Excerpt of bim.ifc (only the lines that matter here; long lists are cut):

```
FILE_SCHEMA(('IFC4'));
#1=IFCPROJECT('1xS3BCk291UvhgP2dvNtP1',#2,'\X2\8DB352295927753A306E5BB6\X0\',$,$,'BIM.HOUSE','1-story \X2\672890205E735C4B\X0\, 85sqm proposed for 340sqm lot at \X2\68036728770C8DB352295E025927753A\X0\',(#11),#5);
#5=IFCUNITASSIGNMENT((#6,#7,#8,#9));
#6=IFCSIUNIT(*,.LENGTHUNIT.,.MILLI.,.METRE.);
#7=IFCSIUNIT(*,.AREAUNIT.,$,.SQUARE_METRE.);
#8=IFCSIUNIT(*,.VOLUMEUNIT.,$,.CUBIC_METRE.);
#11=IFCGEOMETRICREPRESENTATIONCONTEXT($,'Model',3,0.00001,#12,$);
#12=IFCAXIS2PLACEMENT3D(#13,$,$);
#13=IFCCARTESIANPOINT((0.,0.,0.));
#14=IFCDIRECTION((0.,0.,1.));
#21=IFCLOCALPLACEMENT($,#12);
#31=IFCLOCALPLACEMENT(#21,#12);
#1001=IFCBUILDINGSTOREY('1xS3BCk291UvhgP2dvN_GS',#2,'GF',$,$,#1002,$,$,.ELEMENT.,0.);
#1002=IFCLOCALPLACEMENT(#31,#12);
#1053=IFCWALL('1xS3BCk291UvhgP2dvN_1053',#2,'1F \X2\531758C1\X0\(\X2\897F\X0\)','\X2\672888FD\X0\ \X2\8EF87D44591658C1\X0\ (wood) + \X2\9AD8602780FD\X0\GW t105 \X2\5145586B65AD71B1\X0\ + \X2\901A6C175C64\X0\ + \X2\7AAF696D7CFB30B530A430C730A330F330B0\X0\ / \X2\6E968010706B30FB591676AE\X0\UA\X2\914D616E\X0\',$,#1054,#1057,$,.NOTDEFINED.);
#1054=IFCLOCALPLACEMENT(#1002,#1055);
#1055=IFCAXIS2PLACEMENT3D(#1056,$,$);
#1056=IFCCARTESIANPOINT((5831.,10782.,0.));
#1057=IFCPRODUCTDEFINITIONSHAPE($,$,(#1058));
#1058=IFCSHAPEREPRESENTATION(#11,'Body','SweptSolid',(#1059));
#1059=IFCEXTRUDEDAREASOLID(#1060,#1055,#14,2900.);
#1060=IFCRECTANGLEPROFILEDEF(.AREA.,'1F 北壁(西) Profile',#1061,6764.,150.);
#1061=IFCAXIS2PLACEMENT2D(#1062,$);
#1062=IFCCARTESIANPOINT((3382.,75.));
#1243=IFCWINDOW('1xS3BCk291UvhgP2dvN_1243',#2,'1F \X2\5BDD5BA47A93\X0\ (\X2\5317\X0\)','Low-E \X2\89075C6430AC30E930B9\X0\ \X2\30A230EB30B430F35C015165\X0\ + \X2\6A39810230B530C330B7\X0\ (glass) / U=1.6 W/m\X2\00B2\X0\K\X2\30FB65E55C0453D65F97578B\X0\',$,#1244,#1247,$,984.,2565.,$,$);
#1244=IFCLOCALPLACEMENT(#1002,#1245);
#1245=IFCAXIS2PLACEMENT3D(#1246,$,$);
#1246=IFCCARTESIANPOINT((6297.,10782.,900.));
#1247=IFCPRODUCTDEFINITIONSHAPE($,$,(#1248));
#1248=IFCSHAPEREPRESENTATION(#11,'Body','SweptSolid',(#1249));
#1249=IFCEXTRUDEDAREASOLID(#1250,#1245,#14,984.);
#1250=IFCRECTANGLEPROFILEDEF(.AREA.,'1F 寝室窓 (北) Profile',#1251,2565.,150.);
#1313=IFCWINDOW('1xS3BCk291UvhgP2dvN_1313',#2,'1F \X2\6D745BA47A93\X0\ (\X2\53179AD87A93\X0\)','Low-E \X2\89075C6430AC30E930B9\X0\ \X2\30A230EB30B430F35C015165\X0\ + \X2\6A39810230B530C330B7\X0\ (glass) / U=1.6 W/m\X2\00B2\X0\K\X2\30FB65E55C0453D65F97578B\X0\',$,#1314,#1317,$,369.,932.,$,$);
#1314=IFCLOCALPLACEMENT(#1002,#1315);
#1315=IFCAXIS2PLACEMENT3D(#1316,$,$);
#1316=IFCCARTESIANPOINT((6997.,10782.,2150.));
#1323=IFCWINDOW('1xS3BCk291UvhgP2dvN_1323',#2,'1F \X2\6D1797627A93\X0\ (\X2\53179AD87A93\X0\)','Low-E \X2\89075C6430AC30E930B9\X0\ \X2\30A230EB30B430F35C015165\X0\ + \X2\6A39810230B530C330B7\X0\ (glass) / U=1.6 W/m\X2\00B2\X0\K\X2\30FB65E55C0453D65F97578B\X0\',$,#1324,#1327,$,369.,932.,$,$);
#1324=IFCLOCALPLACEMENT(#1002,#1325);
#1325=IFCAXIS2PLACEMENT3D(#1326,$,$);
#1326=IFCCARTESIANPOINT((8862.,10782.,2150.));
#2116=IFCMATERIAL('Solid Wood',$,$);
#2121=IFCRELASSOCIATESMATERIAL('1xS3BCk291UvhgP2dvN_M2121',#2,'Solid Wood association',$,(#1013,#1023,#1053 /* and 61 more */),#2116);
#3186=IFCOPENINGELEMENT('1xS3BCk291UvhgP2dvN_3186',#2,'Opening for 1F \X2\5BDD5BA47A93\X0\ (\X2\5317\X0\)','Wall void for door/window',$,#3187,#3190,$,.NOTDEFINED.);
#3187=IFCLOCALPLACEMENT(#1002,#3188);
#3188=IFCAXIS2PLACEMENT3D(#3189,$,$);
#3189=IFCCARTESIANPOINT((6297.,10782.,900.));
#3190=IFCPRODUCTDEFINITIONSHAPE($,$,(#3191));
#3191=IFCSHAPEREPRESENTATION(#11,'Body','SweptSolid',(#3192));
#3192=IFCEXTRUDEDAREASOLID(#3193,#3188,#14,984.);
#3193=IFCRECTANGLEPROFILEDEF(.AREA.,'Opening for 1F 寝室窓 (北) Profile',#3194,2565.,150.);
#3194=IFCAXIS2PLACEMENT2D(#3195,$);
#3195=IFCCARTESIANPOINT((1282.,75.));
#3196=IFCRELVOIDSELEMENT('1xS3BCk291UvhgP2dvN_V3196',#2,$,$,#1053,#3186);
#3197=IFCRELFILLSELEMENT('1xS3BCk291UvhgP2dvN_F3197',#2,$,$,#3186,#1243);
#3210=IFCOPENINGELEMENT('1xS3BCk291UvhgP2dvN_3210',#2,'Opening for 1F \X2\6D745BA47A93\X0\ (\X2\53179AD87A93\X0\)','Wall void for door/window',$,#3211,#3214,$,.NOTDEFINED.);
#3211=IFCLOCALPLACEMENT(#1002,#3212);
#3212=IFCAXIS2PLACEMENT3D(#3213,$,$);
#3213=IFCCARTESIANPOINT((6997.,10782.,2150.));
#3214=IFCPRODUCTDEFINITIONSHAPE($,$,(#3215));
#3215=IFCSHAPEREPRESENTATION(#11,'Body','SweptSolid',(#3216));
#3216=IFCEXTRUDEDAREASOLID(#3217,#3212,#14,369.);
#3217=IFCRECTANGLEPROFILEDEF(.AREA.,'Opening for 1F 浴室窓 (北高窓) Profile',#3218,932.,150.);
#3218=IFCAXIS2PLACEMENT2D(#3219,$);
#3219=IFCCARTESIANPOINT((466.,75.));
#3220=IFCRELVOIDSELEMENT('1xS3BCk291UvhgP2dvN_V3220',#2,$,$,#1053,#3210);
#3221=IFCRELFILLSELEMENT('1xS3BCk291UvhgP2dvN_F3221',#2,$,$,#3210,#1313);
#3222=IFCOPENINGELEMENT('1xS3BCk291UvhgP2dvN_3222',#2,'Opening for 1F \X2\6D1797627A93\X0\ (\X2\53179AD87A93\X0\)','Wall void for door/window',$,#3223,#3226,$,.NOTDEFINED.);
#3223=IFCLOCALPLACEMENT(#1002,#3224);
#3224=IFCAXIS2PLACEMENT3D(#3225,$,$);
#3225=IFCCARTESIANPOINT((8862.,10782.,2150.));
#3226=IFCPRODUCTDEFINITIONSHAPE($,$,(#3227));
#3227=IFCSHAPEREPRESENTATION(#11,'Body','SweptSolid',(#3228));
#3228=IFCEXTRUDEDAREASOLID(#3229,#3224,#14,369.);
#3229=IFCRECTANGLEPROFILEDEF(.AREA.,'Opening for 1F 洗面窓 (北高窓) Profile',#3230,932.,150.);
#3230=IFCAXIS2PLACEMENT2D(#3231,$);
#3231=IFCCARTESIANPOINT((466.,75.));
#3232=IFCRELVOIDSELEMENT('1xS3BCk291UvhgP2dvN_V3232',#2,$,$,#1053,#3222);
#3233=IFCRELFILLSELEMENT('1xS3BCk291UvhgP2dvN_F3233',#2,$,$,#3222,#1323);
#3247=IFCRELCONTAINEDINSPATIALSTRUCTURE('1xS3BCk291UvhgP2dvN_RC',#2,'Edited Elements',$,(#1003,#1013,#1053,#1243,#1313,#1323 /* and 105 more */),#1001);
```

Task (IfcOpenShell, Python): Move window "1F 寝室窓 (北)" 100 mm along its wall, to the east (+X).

```python
import ifcopenshell
import ifcopenshell.api.geometry
import ifcopenshell.util.placement
import ifcopenshell.util.unit

model = ifcopenshell.open("bim.ifc")
unit_scale = ifcopenshell.util.unit.calculate_unit_scale(model)

window = model.by_guid("1xS3BCk291UvhgP2dvN_1243")
opening = window.FillsVoids[0].RelatingOpeningElement
wall = opening.VoidsElements[0].RelatingBuildingElement

wall_matrix = ifcopenshell.util.placement.get_local_placement(wall.ObjectPlacement)
shift = wall_matrix[:3, 0] * 0.1 / unit_scale
before = ifcopenshell.util.placement.get_local_placement(window.ObjectPlacement)[:3, 3].copy()

# The window is not placed relative to its opening, so move both.
for product in (opening, window):
    matrix = ifcopenshell.util.placement.get_local_placement(product.ObjectPlacement)
    matrix[:3, 3] += shift
    ifcopenshell.api.geometry.edit_object_placement(model, product=product, matrix=matrix, is_si=False)

after = ifcopenshell.util.placement.get_local_placement(window.ObjectPlacement)[:3, 3]
print("window moved by", (after - before).round(3) + 0.0)

model.write("bim_edited.ifc")
```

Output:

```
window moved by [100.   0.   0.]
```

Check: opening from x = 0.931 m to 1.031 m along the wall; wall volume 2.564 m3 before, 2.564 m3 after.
